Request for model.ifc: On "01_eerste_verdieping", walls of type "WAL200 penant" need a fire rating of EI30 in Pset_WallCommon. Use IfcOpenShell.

First a look at what the model holds.

```python
import ifcopenshell
import ifcopenshell.util.element

model = ifcopenshell.open("model.ifc")
print(model.schema)
storey = next(s for s in model.by_type("IfcBuildingStorey") if s.Name == "01_eerste_verdieping")
walls = [e for e in ifcopenshell.util.element.get_decomposition(storey) if e.is_a("IfcWall")]
seen = {}
for e in walls:
    element_type = ifcopenshell.util.element.get_type(e)
    key = (element_type.Name if element_type != e and element_type else None, ifcopenshell.util.element.get_pset(e, "Pset_WallCommon", "FireRating"))
    seen[key] = seen.get(key, 0) + 1
for (name, value), count in sorted(seen.items(), key=str):
    print(count, "x", name, "|", value)
```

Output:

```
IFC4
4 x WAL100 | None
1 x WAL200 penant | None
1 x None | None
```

```python
import ifcopenshell
import ifcopenshell.api.pset
import ifcopenshell.util.element

model = ifcopenshell.open("model.ifc")

storey = next(s for s in model.by_type("IfcBuildingStorey") if s.Name == "01_eerste_verdieping")
walls = [e for e in ifcopenshell.util.element.get_decomposition(storey) if e.is_a("IfcWall")]

count = 0
for e in walls:
    element_type = ifcopenshell.util.element.get_type(e)
    if element_type in (None, e) or element_type.Name != "WAL200 penant":
        continue
    # add_pset returns the element's existing set when there is one.
    pset = ifcopenshell.api.pset.add_pset(model, product=e, name="Pset_WallCommon")
    ifcopenshell.api.pset.edit_pset(model, pset=pset, properties={"FireRating": "EI30"})
    count += 1

print(count, "walls updated")

model.write("model-out.ifc")
```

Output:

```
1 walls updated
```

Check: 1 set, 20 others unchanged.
